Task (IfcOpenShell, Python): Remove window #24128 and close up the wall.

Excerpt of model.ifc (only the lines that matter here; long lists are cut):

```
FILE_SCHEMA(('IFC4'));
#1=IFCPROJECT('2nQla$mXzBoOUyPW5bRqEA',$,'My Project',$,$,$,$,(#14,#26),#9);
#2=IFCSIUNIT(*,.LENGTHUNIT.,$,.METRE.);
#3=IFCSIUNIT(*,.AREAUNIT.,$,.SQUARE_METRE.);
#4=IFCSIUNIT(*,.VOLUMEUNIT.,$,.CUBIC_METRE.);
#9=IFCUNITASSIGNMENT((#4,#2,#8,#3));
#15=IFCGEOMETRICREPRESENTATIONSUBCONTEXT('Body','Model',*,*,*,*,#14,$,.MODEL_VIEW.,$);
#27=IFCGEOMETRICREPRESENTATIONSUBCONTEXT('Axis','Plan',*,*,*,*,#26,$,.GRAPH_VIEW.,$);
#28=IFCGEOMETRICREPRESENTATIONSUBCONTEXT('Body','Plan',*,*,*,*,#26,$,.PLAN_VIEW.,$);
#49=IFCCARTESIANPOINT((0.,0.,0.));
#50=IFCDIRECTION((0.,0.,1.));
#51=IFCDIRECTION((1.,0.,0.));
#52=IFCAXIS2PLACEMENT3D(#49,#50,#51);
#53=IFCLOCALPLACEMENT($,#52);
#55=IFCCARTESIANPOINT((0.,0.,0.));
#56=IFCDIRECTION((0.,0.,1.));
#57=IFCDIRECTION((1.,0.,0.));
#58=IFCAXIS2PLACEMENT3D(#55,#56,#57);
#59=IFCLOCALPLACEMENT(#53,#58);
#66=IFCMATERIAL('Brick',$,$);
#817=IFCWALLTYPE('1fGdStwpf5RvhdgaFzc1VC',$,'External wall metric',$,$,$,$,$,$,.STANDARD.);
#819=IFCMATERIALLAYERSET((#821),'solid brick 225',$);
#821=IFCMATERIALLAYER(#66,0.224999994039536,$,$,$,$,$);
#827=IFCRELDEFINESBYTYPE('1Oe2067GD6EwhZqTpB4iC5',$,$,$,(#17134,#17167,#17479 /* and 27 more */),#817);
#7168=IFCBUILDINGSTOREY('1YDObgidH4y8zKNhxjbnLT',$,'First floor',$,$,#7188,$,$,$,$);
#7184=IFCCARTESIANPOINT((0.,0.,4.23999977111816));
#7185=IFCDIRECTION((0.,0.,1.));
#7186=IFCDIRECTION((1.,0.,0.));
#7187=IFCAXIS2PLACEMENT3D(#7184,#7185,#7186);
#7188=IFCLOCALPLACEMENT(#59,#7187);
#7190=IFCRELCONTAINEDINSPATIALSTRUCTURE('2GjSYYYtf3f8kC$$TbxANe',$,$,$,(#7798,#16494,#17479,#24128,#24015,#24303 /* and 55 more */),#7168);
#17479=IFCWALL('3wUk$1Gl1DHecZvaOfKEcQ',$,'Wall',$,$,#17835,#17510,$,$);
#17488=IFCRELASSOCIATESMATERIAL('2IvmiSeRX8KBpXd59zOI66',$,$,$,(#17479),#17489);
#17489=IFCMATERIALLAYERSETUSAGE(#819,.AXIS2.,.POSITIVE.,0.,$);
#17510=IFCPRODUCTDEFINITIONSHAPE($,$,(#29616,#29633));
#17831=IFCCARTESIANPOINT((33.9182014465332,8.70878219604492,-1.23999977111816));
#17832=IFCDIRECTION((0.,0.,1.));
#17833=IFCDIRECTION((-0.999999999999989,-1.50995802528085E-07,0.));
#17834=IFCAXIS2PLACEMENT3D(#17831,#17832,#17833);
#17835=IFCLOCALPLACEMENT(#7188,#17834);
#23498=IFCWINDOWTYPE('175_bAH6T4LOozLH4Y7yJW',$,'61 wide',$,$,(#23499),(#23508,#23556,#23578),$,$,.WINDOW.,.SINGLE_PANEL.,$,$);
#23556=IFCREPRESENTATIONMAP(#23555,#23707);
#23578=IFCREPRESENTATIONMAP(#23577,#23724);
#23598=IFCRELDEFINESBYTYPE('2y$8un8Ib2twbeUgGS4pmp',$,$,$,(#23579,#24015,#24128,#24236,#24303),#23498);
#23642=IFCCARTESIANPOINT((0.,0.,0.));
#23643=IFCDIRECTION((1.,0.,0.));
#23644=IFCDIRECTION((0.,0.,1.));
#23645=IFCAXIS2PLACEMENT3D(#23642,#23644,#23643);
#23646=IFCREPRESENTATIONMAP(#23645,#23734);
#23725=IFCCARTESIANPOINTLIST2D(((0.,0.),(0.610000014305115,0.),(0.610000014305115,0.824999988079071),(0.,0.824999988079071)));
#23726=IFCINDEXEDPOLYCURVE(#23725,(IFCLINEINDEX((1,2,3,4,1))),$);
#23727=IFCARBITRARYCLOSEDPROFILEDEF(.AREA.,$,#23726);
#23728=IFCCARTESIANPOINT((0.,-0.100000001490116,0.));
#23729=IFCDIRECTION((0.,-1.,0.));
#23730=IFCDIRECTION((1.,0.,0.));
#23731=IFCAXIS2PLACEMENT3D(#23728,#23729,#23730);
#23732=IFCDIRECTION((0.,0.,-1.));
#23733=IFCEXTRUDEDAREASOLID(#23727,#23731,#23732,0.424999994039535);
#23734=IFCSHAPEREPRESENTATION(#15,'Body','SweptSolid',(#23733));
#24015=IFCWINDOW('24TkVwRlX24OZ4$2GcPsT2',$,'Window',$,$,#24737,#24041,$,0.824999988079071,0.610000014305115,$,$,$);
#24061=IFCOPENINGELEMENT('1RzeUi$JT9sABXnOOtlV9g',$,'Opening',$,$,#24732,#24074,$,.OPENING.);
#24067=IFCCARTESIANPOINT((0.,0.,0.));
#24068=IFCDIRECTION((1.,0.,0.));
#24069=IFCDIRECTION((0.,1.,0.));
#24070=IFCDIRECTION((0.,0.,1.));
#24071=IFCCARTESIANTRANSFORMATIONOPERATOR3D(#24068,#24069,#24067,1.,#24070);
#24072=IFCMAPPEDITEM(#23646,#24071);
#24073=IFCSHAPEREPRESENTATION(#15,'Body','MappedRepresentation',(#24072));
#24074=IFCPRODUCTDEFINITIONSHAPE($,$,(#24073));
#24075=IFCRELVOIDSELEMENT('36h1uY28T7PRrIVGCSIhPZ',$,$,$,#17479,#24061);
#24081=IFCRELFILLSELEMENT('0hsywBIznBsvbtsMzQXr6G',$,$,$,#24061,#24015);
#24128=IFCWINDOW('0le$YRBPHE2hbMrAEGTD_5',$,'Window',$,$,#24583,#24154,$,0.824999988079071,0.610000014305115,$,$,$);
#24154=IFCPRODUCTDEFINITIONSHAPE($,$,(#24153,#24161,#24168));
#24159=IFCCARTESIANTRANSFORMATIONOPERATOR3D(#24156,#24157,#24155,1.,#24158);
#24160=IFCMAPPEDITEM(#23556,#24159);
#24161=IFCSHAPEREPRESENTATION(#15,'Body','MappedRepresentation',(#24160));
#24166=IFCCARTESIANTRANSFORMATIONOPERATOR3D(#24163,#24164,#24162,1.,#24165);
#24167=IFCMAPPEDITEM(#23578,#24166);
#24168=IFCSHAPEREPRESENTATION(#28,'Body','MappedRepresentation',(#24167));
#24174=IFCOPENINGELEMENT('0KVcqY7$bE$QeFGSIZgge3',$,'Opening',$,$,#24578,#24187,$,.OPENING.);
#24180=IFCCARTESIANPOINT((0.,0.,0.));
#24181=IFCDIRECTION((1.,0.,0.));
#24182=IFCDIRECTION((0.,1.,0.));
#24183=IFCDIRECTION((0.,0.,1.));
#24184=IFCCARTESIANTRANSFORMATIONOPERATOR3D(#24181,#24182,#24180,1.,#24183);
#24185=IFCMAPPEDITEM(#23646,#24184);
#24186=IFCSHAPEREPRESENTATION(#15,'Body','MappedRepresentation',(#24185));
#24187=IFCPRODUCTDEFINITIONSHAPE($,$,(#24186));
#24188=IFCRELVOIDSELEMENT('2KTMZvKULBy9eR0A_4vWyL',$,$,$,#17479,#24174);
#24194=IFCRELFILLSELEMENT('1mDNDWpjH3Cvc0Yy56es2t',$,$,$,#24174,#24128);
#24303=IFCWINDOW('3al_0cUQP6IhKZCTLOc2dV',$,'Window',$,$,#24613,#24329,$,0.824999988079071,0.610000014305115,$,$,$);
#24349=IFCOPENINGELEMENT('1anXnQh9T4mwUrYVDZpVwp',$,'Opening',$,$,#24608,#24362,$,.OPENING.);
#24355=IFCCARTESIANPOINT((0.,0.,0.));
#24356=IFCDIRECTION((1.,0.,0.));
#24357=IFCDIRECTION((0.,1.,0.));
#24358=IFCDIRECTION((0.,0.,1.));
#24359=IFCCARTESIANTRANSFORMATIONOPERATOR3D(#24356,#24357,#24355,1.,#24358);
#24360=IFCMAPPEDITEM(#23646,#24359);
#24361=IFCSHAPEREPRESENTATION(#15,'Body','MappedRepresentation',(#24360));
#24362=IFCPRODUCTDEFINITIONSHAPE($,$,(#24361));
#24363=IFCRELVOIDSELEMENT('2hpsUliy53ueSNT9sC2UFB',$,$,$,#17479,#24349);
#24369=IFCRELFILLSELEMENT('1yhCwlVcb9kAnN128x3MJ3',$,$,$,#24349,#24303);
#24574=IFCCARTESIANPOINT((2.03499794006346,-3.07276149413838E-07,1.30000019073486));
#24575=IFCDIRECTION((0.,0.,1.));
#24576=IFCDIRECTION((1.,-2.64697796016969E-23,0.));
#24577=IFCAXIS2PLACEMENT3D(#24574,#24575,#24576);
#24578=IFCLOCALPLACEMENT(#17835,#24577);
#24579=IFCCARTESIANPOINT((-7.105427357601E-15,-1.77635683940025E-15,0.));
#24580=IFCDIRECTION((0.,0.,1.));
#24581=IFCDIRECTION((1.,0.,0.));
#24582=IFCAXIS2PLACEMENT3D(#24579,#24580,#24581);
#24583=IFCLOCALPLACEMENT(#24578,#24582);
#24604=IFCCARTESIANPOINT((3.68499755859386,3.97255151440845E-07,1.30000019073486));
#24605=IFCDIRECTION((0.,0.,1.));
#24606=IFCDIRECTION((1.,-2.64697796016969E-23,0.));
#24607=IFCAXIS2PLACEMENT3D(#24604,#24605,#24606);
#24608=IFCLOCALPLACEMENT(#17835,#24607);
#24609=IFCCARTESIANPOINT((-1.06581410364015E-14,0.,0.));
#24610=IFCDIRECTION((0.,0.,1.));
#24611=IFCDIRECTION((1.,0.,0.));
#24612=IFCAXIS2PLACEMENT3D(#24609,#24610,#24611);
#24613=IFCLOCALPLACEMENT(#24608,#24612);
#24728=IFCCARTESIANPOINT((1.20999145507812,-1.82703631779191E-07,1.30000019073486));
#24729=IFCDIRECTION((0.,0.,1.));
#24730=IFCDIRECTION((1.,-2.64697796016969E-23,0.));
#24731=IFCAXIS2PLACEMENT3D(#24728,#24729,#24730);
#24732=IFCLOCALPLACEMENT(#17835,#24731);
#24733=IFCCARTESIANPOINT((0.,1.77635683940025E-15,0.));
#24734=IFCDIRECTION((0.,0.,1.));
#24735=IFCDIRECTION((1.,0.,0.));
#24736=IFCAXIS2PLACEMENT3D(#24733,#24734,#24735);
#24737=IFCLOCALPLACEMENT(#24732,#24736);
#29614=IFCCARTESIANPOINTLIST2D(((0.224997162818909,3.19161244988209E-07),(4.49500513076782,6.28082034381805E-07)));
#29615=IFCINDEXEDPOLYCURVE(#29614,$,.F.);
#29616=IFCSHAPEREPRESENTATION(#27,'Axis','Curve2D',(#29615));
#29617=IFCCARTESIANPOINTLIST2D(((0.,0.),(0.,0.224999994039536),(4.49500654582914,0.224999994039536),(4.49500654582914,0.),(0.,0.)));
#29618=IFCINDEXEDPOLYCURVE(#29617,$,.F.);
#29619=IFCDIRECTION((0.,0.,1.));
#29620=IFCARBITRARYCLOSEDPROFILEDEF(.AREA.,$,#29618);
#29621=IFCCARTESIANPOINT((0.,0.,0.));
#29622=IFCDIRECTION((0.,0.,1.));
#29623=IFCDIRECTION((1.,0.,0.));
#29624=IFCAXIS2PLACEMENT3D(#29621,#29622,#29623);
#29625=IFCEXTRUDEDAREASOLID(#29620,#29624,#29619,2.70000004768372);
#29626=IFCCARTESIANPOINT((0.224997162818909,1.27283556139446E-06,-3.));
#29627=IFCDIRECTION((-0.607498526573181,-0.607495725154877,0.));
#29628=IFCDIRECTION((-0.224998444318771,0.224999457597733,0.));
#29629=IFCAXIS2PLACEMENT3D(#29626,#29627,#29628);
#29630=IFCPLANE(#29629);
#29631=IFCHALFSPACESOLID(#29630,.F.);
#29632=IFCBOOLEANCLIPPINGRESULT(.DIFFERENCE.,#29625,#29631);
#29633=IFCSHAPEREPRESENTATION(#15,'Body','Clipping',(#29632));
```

```python
import ifcopenshell
import ifcopenshell.api.feature
import ifcopenshell.api.root
import ifcopenshell.geom
import ifcopenshell.util.shape

model = ifcopenshell.open("model.ifc")
settings = ifcopenshell.geom.settings()


def volume(element):
    """Net volume in cubic metres, openings subtracted."""
    shape = ifcopenshell.geom.create_shape(settings, element)
    return ifcopenshell.util.shape.get_volume(shape.geometry)


window = model.by_guid("0le$YRBPHE2hbMrAEGTD_5")
opening = window.FillsVoids[0].RelatingOpeningElement
wall = opening.VoidsElements[0].RelatingBuildingElement
before = volume(wall)

ifcopenshell.api.root.remove_product(model, product=window)
ifcopenshell.api.feature.remove_feature(model, feature=opening)

after = volume(wall)

print(f"wall volume {before:.3f} -> {after:.3f} m3")

model.write("model_rev.ifc")
```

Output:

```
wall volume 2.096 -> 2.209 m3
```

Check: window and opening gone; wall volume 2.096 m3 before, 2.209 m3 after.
